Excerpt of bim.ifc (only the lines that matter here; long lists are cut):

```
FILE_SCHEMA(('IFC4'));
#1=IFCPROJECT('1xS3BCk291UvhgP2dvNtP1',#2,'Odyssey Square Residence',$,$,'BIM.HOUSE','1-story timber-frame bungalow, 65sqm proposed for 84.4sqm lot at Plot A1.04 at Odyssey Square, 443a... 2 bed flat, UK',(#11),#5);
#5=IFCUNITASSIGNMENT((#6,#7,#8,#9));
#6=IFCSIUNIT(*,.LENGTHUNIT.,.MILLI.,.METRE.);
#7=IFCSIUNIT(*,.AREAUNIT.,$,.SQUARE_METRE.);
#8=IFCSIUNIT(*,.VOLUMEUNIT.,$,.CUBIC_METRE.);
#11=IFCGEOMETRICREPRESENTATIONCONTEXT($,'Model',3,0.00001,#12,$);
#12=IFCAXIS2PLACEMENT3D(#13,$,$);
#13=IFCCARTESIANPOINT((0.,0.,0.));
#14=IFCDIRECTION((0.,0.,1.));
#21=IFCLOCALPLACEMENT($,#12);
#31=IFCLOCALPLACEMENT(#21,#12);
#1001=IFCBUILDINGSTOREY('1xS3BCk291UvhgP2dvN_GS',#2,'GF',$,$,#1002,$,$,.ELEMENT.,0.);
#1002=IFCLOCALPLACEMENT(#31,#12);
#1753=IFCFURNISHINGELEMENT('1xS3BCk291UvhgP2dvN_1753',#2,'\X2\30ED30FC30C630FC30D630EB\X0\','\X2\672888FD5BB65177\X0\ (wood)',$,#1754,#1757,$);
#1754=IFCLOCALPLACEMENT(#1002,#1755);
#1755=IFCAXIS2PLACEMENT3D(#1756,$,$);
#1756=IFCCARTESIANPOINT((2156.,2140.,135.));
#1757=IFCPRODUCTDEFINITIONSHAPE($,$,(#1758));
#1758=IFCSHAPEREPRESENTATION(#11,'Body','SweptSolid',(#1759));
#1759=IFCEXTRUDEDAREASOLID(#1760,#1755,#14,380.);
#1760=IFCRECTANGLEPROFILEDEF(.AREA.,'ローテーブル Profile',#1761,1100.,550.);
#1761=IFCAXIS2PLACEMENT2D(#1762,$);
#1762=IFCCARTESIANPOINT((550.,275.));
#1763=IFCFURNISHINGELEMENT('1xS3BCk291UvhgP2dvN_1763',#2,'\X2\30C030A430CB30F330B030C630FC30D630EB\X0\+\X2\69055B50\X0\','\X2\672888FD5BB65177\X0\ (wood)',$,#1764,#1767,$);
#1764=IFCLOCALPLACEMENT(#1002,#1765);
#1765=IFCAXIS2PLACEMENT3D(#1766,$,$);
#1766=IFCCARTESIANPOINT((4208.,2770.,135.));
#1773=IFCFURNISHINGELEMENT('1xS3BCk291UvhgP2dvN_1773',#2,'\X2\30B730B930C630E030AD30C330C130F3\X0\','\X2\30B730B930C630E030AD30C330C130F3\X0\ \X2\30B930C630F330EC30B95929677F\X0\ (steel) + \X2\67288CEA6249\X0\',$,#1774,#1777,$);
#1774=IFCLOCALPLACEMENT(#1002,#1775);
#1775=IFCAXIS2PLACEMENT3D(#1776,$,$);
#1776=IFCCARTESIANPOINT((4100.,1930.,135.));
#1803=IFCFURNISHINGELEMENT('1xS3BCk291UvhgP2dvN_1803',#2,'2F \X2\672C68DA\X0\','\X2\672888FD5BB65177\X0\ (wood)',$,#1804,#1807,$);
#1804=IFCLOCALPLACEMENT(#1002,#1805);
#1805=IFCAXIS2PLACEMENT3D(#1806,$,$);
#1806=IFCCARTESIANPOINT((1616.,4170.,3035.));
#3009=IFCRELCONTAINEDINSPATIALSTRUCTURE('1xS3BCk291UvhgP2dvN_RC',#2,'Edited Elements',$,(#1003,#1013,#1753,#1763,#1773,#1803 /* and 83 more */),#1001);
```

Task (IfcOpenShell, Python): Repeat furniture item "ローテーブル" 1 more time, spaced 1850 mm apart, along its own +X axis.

```python
import ifcopenshell
import ifcopenshell.api.geometry
import ifcopenshell.api.root
import ifcopenshell.util.element
import ifcopenshell.util.placement
import ifcopenshell.util.unit

model = ifcopenshell.open("bim.ifc")
unit_scale = ifcopenshell.util.unit.calculate_unit_scale(model)


def reuse_history(source, copy):
    """copy_class also copies each property set's owner history, people and application; keep the originals."""
    for rel in copy.IsDefinedBy:
        if rel.is_a("IfcRelDefinesByProperties") and (history := rel.RelatingPropertyDefinition.OwnerHistory):
            rel.RelatingPropertyDefinition.OwnerHistory = source.OwnerHistory
            ifcopenshell.util.element.remove_deep2(model, history)


source = model.by_guid("1xS3BCk291UvhgP2dvN_1753")
base = ifcopenshell.util.placement.get_local_placement(source.ObjectPlacement)
step = base[:3, 0] * 1.85 / unit_scale

for i in range(1, 2):
    copy = ifcopenshell.api.root.copy_class(model, product=source)
    copy.Representation = ifcopenshell.util.element.copy_deep(
        model, source.Representation, exclude=["IfcGeometricRepresentationContext", "IfcRepresentationMap"]
    )
    reuse_history(source, copy)
    matrix = base.copy()
    matrix[:3, 3] += i * step
    print("added at", matrix[:3, 3].round(3) + 0.0)
    ifcopenshell.api.geometry.edit_object_placement(model, product=copy, matrix=matrix, is_si=False)

model.write("bim_updated.ifc")
```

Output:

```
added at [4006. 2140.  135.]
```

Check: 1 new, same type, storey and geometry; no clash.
